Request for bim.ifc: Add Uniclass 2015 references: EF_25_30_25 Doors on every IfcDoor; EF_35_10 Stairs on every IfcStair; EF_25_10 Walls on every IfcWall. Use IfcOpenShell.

First a look at what the model holds.

```python
import ifcopenshell

model = ifcopenshell.open("bim.ifc")
print(model.schema)
print("classifications:", [c.Name for c in model.by_type("IfcClassification")])
for ifc_class in ("IfcDoor", "IfcRoof", "IfcStair", "IfcWall", "IfcWindow"):
    print(ifc_class, len(model.by_type(ifc_class)))
```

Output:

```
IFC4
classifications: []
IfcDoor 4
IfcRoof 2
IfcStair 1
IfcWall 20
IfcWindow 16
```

```python
import ifcopenshell
import ifcopenshell.api.classification

model = ifcopenshell.open("bim.ifc")

system = ifcopenshell.api.classification.add_classification(model, classification="Uniclass 2015")

codes = {
    "IfcDoor": ("EF_25_30_25", "Doors"),
    "IfcStair": ("EF_35_10", "Stairs"),
    "IfcWall": ("EF_25_10", "Walls"),
}
for ifc_class, (code, name) in codes.items():
    products = model.by_type(ifc_class)
    ifcopenshell.api.classification.add_reference(
        model, products=products, classification=system, identification=code, name=name
    )
    print(code, len(products))

model.write("bim_rev.ifc")
```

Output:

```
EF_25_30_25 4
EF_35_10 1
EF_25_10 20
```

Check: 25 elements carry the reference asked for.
